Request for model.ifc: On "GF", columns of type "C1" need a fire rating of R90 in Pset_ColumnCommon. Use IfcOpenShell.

First a look at what the model holds.

```python
import ifcopenshell
import ifcopenshell.util.element

model = ifcopenshell.open("model.ifc")
print(model.schema)
storey = next(s for s in model.by_type("IfcBuildingStorey") if s.Name == "GF")
columns = [e for e in ifcopenshell.util.element.get_decomposition(storey) if e.is_a("IfcColumn")]
seen = {}
for e in columns:
    element_type = ifcopenshell.util.element.get_type(e)
    key = (element_type.Name if element_type != e and element_type else None, ifcopenshell.util.element.get_pset(e, "Pset_ColumnCommon", "FireRating"))
    seen[key] = seen.get(key, 0) + 1
for (name, value), count in sorted(seen.items(), key=str):
    print(count, "x", name, "|", value)
```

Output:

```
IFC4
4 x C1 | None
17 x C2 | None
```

```python
import ifcopenshell
import ifcopenshell.api.pset
import ifcopenshell.util.element

model = ifcopenshell.open("model.ifc")

storey = next(s for s in model.by_type("IfcBuildingStorey") if s.Name == "GF")
columns = [e for e in ifcopenshell.util.element.get_decomposition(storey) if e.is_a("IfcColumn")]

count = 0
for e in columns:
    element_type = ifcopenshell.util.element.get_type(e)
    if element_type in (None, e) or element_type.Name != "C1":
        continue
    # add_pset returns the element's existing set when there is one.
    pset = ifcopenshell.api.pset.add_pset(model, product=e, name="Pset_ColumnCommon")
    ifcopenshell.api.pset.edit_pset(model, pset=pset, properties={"FireRating": "R90"})
    count += 1

print(count, "columns updated")

model.write("model_v2.ifc")
```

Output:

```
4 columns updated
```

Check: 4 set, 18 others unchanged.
